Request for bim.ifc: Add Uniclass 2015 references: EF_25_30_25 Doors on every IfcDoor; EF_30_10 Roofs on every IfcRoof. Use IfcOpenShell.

First a look at what the model holds.

```python
import ifcopenshell

model = ifcopenshell.open("bim.ifc")
print(model.schema)
print("classifications:", [c.Name for c in model.by_type("IfcClassification")])
for ifc_class in ("IfcDoor", "IfcRoof", "IfcStair", "IfcWall", "IfcWindow"):
    print(ifc_class, len(model.by_type(ifc_class)))
```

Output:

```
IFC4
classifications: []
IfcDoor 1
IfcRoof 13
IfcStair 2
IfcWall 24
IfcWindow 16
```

```python
import ifcopenshell
import ifcopenshell.api.classification

model = ifcopenshell.open("bim.ifc")

system = ifcopenshell.api.classification.add_classification(model, classification="Uniclass 2015")

codes = {
    "IfcDoor": ("EF_25_30_25", "Doors"),
    "IfcRoof": ("EF_30_10", "Roofs"),
}
for ifc_class, (code, name) in codes.items():
    products = model.by_type(ifc_class)
    ifcopenshell.api.classification.add_reference(
        model, products=products, classification=system, identification=code, name=name
    )
    print(code, len(products))

model.write("bim_edited.ifc")
```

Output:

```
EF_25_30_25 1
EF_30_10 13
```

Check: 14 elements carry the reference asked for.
